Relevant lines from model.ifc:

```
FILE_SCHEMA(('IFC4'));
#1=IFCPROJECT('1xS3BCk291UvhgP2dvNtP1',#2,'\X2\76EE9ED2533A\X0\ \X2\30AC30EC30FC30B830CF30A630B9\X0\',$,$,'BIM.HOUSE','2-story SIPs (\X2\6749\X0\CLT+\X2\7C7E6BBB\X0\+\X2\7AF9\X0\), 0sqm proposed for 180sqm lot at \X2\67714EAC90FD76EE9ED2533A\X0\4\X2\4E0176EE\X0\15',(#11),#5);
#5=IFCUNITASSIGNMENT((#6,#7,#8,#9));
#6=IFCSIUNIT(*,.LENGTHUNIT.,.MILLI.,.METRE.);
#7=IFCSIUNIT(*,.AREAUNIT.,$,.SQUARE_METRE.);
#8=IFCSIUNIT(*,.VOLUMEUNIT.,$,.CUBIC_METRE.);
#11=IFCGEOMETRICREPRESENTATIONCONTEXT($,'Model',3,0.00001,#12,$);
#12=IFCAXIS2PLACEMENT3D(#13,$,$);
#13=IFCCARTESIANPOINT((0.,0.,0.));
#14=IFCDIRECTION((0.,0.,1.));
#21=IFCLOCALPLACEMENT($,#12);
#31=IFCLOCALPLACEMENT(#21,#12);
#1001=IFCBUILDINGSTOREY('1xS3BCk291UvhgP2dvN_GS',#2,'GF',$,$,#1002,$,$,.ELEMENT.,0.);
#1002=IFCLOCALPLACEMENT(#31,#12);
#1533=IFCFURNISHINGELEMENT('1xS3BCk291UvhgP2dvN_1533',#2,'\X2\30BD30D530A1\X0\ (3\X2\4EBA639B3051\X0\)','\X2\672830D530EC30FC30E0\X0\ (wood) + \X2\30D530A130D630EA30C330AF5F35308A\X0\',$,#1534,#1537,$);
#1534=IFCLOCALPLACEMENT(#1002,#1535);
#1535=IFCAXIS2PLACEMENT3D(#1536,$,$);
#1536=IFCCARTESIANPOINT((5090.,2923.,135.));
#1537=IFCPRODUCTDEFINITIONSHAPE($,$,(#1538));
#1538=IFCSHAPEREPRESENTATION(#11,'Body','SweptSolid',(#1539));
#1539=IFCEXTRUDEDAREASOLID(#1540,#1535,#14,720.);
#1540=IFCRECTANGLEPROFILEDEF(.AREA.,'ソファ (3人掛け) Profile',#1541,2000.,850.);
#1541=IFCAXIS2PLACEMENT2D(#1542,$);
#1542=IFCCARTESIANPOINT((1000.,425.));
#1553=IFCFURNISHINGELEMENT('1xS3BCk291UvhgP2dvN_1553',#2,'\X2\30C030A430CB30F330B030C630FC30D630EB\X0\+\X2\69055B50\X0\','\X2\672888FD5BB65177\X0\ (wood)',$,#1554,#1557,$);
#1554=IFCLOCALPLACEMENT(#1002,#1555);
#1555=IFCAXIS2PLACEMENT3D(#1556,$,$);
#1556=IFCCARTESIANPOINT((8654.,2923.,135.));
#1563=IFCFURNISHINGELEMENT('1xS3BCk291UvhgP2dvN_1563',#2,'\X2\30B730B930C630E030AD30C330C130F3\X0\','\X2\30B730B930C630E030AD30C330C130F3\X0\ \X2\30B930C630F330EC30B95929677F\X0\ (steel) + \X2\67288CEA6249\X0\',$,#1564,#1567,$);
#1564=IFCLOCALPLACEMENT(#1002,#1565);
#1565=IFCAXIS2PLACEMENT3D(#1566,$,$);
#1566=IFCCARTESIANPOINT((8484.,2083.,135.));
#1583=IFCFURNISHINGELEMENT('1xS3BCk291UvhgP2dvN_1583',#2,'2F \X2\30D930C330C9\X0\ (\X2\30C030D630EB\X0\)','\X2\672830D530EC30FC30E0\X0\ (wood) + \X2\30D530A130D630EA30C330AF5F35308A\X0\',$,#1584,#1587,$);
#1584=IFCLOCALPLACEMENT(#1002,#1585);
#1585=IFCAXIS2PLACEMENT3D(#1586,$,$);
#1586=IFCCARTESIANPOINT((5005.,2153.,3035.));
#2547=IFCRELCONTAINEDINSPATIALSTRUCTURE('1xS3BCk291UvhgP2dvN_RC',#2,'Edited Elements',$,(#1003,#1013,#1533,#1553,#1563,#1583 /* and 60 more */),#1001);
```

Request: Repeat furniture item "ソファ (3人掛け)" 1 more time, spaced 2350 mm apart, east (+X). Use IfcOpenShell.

```python
import numpy as np
import ifcopenshell
import ifcopenshell.api.geometry
import ifcopenshell.api.root
import ifcopenshell.util.element
import ifcopenshell.util.placement

model = ifcopenshell.open("model.ifc")


def reuse_history(source, copy):
    """copy_class also copies each property set's owner history, people and application; keep the originals."""
    for rel in copy.IsDefinedBy:
        if rel.is_a("IfcRelDefinesByProperties") and (history := rel.RelatingPropertyDefinition.OwnerHistory):
            rel.RelatingPropertyDefinition.OwnerHistory = source.OwnerHistory
            ifcopenshell.util.element.remove_deep2(model, history)


source = model.by_guid("1xS3BCk291UvhgP2dvN_1533")
base = ifcopenshell.util.placement.get_local_placement(source.ObjectPlacement)
step = np.array([1.0, 0.0, 0.0]) * 2350.0

for i in range(1, 2):
    copy = ifcopenshell.api.root.copy_class(model, product=source)
    copy.Representation = ifcopenshell.util.element.copy_deep(
        model, source.Representation, exclude=["IfcGeometricRepresentationContext", "IfcRepresentationMap"]
    )
    reuse_history(source, copy)
    matrix = base.copy()
    matrix[:3, 3] += i * step
    print("added at", matrix[:3, 3].round(3) + 0.0)
    ifcopenshell.api.geometry.edit_object_placement(model, product=copy, matrix=matrix, is_si=False)

model.write("model_updated.ifc")
```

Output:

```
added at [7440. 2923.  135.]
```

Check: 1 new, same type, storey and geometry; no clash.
